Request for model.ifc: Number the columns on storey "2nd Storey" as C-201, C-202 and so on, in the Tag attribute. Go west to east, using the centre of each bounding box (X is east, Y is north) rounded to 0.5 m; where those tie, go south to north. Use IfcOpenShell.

First a look at what the model holds.

```python
import ifcopenshell
import ifcopenshell.util.element
import ifcopenshell.util.placement

model = ifcopenshell.open("model.ifc")
print(model.schema)
storey = next(s for s in model.by_type("IfcBuildingStorey") if s.Name == "2nd Storey")
columns = [e for e in ifcopenshell.util.element.get_decomposition(storey) if e.is_a("IfcColumn")]
for e in sorted(columns, key=lambda e: e.id()):
    origin = ifcopenshell.util.placement.get_local_placement(e.ObjectPlacement)[:3, 3]
    print(e.id(), e.Tag, e.Name, origin.round(2) + 0.0, sep=" | ")
```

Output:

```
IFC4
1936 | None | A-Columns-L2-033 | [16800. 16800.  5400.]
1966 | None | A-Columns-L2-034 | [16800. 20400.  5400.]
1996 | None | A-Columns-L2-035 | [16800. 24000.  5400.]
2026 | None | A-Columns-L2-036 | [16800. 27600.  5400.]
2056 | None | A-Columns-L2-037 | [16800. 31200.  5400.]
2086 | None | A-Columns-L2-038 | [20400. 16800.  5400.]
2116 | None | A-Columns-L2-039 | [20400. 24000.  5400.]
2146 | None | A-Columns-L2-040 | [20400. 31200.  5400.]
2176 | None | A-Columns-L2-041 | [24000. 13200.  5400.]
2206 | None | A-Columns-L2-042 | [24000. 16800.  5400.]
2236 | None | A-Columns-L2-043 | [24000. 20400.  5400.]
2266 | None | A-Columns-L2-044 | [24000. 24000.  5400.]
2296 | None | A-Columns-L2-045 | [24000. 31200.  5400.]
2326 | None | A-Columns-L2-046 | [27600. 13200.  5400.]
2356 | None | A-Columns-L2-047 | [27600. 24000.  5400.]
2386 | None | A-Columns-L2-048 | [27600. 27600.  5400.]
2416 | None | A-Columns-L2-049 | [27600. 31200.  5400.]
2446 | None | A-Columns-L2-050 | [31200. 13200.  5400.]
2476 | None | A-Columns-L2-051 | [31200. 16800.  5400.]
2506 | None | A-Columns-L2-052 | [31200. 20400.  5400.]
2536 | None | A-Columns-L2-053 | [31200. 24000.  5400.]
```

```python
import ifcopenshell
import ifcopenshell.geom
import ifcopenshell.util.element
import ifcopenshell.util.shape

model = ifcopenshell.open("model.ifc")
settings = ifcopenshell.geom.settings()
settings.set("use-world-coords", True)


def centre(element):
    shape = ifcopenshell.geom.create_shape(settings, element)
    return ifcopenshell.util.shape.get_bbox_centroid(shape.geometry)


storey = next(s for s in model.by_type("IfcBuildingStorey") if s.Name == "2nd Storey")
columns = [e for e in ifcopenshell.util.element.get_decomposition(storey) if e.is_a("IfcColumn")]

# Insertion points can sit at a corner or the storey origin, so sort by the geometry (in metres).
centres = {e: centre(e) for e in columns}
columns.sort(key=lambda e: (round(centres[e][0] / 0.5), centres[e][1]))

for i, e in enumerate(columns, start=1):
    number = f"C-2{i:02d}"
    e.Tag = number
    print(e.id(), number)

model.write("model_edited.ifc")
```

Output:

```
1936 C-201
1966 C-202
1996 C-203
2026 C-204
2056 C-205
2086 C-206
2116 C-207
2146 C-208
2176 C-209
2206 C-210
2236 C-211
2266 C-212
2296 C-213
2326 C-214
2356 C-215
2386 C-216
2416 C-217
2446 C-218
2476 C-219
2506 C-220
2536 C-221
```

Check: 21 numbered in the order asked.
